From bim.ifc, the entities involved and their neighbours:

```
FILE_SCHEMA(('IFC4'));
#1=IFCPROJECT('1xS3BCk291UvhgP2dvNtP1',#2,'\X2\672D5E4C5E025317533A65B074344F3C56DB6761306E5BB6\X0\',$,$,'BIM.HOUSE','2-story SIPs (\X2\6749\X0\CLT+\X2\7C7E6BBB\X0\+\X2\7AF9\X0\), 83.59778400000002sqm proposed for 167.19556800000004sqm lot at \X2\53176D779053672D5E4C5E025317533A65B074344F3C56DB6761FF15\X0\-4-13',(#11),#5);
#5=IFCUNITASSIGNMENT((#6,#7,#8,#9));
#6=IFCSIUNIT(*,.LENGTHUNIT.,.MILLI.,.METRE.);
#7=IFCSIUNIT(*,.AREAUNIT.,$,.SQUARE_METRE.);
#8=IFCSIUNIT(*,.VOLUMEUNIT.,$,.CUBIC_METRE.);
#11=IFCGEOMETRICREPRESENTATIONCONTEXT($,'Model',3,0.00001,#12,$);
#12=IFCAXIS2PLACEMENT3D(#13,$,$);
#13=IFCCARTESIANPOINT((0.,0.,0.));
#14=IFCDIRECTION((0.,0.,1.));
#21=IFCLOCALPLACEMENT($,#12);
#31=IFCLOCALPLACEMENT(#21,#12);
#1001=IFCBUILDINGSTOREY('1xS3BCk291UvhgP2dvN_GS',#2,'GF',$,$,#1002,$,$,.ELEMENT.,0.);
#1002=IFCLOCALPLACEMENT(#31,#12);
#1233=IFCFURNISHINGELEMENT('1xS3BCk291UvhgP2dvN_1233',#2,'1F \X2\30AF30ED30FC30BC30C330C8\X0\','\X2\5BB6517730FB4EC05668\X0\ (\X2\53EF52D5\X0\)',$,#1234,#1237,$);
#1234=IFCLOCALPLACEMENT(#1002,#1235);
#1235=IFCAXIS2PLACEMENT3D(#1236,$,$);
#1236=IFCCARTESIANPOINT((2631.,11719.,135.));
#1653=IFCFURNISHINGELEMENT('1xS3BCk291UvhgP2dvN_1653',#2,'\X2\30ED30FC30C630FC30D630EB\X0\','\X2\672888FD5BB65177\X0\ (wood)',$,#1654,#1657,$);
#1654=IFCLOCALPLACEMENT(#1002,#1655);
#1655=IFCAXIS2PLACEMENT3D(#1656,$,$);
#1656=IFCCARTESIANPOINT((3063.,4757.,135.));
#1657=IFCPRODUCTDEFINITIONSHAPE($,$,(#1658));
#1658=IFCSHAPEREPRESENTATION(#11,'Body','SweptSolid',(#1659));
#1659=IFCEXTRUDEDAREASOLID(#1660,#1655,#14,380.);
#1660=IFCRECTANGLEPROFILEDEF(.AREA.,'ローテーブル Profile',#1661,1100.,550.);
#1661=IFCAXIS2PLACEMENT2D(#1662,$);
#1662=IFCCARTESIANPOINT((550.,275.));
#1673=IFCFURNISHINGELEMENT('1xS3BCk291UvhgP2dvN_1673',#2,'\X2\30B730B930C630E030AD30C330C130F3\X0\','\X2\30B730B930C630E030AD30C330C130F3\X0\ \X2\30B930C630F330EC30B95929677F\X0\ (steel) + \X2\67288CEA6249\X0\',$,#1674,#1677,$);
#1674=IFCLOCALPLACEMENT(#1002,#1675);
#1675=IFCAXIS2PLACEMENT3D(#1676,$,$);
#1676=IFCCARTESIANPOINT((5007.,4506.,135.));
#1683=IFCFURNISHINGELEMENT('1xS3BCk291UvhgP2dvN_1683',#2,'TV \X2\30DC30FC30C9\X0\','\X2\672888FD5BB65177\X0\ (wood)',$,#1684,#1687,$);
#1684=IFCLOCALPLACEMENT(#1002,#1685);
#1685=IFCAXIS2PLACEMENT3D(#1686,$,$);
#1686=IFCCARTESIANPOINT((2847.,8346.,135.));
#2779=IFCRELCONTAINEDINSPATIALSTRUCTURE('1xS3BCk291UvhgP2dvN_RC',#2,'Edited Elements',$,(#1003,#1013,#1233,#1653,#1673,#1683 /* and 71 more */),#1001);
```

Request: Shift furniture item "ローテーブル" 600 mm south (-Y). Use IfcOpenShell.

```python
import ifcopenshell
import ifcopenshell.api.geometry
import ifcopenshell.util.placement

model = ifcopenshell.open("bim.ifc")

item = model.by_guid("1xS3BCk291UvhgP2dvN_1653")
matrix = ifcopenshell.util.placement.get_local_placement(item.ObjectPlacement)
matrix[1, 3] -= 600.0
ifcopenshell.api.geometry.edit_object_placement(model, product=item, matrix=matrix, is_si=False)

print(ifcopenshell.util.placement.get_local_placement(item.ObjectPlacement).round(3) + 0.0)

model.write("bim-out.ifc")
```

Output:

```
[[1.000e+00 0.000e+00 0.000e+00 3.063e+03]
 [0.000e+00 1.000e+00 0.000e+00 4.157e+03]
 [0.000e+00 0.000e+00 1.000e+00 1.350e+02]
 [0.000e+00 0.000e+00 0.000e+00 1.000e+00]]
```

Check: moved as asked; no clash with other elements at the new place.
